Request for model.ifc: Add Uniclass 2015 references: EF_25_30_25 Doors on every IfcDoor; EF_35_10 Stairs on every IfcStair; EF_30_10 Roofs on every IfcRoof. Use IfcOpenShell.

First a look at what the model holds.

```python
import ifcopenshell

model = ifcopenshell.open("model.ifc")
print(model.schema)
print("classifications:", [c.Name for c in model.by_type("IfcClassification")])
for ifc_class in ("IfcDoor", "IfcRoof", "IfcStair", "IfcWall", "IfcWindow"):
    print(ifc_class, len(model.by_type(ifc_class)))
```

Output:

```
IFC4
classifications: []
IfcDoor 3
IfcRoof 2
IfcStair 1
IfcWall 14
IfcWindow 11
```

```python
import ifcopenshell
import ifcopenshell.api.classification

model = ifcopenshell.open("model.ifc")

system = ifcopenshell.api.classification.add_classification(model, classification="Uniclass 2015")

codes = {
    "IfcDoor": ("EF_25_30_25", "Doors"),
    "IfcStair": ("EF_35_10", "Stairs"),
    "IfcRoof": ("EF_30_10", "Roofs"),
}
for ifc_class, (code, name) in codes.items():
    products = model.by_type(ifc_class)
    ifcopenshell.api.classification.add_reference(
        model, products=products, classification=system, identification=code, name=name
    )
    print(code, len(products))

model.write("model_rev.ifc")
```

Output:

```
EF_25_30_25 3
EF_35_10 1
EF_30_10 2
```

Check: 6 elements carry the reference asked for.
